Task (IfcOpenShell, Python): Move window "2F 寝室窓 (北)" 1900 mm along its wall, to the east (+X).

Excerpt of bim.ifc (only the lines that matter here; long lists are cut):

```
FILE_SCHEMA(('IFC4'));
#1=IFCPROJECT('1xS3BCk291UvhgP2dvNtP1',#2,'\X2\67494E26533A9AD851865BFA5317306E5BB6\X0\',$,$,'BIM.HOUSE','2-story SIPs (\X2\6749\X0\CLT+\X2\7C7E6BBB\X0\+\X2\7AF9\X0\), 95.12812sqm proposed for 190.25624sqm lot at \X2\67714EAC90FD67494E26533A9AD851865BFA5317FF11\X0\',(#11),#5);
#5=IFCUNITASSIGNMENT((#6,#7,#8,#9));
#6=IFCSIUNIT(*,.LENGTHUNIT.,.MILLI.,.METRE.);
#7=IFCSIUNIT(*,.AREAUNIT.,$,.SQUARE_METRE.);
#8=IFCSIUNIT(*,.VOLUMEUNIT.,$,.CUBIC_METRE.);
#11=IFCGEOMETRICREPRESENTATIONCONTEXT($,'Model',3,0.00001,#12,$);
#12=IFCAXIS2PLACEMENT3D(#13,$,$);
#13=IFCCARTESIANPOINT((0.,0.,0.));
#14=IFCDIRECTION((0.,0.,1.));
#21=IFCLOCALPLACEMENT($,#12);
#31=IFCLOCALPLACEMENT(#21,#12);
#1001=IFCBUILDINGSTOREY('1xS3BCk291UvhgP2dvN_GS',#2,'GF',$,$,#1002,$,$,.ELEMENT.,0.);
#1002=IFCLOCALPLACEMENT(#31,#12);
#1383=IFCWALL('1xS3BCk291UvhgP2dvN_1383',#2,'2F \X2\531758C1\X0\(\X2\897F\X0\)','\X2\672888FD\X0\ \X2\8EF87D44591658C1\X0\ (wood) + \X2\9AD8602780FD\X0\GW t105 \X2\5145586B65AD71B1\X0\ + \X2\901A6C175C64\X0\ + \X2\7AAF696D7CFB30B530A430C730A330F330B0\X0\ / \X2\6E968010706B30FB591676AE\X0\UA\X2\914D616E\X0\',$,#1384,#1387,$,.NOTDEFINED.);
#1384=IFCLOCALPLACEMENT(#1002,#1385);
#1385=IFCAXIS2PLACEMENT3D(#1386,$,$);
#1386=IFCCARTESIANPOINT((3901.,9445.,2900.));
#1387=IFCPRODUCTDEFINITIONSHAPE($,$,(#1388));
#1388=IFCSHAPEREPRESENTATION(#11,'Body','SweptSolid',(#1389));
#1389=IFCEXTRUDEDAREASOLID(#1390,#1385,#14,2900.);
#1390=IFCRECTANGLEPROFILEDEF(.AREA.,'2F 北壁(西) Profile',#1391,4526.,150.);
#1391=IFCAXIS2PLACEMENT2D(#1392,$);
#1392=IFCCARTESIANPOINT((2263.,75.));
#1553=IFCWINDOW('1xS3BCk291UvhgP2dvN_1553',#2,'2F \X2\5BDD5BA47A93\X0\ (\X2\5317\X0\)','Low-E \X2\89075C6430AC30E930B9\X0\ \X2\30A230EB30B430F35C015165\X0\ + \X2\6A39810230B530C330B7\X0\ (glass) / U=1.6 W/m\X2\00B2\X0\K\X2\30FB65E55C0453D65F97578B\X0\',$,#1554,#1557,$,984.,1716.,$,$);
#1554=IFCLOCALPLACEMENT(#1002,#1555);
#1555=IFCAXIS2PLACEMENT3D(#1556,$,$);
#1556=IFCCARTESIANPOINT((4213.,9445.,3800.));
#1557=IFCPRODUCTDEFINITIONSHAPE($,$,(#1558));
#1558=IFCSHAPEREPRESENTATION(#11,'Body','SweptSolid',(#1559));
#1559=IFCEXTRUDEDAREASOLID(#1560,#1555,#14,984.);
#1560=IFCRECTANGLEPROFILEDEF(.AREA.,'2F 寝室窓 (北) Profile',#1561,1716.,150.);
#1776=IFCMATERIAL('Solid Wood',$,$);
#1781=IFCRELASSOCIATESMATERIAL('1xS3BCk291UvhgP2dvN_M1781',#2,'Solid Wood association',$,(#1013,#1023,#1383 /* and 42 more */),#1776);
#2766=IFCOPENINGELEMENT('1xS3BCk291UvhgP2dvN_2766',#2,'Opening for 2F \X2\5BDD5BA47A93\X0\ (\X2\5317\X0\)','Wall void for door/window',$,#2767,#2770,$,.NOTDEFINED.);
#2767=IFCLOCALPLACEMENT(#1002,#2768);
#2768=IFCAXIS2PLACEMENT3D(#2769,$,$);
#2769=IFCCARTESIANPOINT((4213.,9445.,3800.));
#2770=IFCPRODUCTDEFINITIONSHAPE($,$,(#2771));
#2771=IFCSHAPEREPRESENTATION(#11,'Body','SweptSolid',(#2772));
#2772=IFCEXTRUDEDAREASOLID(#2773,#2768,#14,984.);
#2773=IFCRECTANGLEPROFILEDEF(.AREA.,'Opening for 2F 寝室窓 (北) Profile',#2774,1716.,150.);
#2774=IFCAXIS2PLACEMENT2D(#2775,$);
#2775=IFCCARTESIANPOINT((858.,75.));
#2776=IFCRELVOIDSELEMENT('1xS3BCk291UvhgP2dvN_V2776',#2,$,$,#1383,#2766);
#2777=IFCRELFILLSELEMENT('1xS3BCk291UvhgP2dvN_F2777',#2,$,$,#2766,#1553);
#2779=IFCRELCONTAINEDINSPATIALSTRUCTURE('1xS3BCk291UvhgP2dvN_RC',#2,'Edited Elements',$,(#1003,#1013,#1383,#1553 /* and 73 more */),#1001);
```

```python
import ifcopenshell
import ifcopenshell.api.geometry
import ifcopenshell.util.placement
import ifcopenshell.util.unit

model = ifcopenshell.open("bim.ifc")
unit_scale = ifcopenshell.util.unit.calculate_unit_scale(model)

window = model.by_guid("1xS3BCk291UvhgP2dvN_1553")
opening = window.FillsVoids[0].RelatingOpeningElement
wall = opening.VoidsElements[0].RelatingBuildingElement

wall_matrix = ifcopenshell.util.placement.get_local_placement(wall.ObjectPlacement)
shift = wall_matrix[:3, 0] * 1.9 / unit_scale
before = ifcopenshell.util.placement.get_local_placement(window.ObjectPlacement)[:3, 3].copy()

# The window is not placed relative to its opening, so move both.
for product in (opening, window):
    matrix = ifcopenshell.util.placement.get_local_placement(product.ObjectPlacement)
    matrix[:3, 3] += shift
    ifcopenshell.api.geometry.edit_object_placement(model, product=product, matrix=matrix, is_si=False)

after = ifcopenshell.util.placement.get_local_placement(window.ObjectPlacement)[:3, 3]
print("window moved by", (after - before).round(3) + 0.0)

model.write("bim_updated.ifc")
```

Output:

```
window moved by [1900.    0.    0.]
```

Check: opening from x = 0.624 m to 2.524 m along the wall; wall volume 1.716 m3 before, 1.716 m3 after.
